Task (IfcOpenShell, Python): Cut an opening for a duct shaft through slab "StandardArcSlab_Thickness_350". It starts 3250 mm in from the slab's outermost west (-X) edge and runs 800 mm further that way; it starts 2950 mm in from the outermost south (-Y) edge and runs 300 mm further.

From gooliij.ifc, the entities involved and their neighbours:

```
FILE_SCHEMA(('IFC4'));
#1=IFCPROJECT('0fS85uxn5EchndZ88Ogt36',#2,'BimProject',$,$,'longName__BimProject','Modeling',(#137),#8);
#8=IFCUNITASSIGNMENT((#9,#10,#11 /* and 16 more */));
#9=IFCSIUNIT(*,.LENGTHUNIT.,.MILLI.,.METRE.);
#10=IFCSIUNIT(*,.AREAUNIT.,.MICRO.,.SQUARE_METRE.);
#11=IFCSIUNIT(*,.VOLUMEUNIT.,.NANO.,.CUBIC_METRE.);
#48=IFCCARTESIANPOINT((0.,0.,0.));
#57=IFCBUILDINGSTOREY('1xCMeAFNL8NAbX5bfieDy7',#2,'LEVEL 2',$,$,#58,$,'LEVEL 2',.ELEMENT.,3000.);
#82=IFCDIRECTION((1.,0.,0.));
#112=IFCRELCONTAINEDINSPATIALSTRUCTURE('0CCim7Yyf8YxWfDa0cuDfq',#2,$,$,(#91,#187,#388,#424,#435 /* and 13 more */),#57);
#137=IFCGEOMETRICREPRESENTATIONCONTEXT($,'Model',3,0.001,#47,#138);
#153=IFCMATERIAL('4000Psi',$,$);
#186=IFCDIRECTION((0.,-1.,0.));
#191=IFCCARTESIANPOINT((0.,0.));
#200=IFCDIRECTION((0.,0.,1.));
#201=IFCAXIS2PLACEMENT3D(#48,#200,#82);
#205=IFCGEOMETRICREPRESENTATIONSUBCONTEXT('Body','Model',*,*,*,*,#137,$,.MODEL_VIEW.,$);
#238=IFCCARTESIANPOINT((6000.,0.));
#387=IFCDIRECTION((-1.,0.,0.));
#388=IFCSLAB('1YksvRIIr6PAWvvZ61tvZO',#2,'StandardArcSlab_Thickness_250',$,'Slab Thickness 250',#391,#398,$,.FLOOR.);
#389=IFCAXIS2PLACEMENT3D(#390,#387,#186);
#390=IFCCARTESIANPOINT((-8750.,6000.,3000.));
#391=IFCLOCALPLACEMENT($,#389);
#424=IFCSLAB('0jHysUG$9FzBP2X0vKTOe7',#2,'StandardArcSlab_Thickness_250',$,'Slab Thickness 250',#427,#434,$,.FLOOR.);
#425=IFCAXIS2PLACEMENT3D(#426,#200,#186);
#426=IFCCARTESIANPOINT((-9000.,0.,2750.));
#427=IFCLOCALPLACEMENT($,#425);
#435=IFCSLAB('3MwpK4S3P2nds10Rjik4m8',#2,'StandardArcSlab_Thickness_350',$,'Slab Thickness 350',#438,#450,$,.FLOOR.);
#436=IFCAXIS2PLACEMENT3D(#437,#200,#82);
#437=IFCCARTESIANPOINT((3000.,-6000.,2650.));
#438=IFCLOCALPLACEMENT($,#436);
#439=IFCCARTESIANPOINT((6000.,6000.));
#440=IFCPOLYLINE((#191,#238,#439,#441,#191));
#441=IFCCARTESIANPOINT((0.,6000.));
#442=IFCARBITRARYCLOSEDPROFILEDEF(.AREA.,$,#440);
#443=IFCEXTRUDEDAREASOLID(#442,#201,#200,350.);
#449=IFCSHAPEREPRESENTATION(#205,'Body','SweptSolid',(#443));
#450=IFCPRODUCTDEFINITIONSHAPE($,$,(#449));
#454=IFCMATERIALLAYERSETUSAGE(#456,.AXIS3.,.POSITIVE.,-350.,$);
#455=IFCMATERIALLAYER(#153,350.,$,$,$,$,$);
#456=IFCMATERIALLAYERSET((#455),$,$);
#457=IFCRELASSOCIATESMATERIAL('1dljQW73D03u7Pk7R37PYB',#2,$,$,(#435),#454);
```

```python
import numpy as np
import ifcopenshell
import ifcopenshell.api.feature
import ifcopenshell.api.geometry
import ifcopenshell.api.root
import ifcopenshell.geom
import ifcopenshell.util.placement
import ifcopenshell.util.representation
import ifcopenshell.util.shape
import ifcopenshell.util.unit

model = ifcopenshell.open("gooliij.ifc")
unit_scale = ifcopenshell.util.unit.calculate_unit_scale(model)
settings = ifcopenshell.geom.settings()


def volume(element):
    """Net volume in cubic metres, openings subtracted."""
    shape = ifcopenshell.geom.create_shape(settings, element)
    return ifcopenshell.util.shape.get_volume(shape.geometry)


slab = model.by_guid("3MwpK4S3P2nds10Rjik4m8")
before = volume(slab)

# Extent in the slab's own axes, in metres. The edges named are its -X and -Y sides.
slab_shape = ifcopenshell.geom.create_shape(settings, slab)
vertices = ifcopenshell.util.shape.get_vertices(slab_shape.geometry)
x_min, y_min, bottom = vertices.min(axis=0)
top = vertices[:, 2].max()

opening = ifcopenshell.api.root.create_entity(model, ifc_class="IfcOpeningElement", name="Duct shaft opening", predefined_type="OPENING")
context = ifcopenshell.util.representation.get_context(model, "Model", "Body", "MODEL_VIEW")
width, depth = 0.8, 0.3
outline = [(0.0, 0.0), (width, 0.0), (width, depth), (0.0, depth), (0.0, 0.0)]
# Overshoot both faces by 50 mm so the cut is clean.
shape = ifcopenshell.api.geometry.add_slab_representation(
    model, context=context, depth=top - bottom + 0.1, polyline=outline
)
ifcopenshell.api.geometry.assign_representation(model, product=opening, representation=shape)

matrix = ifcopenshell.util.placement.get_local_placement(slab.ObjectPlacement)
matrix[:, 3] = matrix @ np.append(np.array([x_min + 3.25, y_min + 2.95, bottom - 0.05]) / unit_scale, 1.0)
ifcopenshell.api.geometry.edit_object_placement(model, product=opening, matrix=matrix, is_si=False)
ifcopenshell.api.feature.add_feature(model, feature=opening, element=slab)

after = volume(slab)

print(f"slab volume {before:.3f} -> {after:.3f} m3")

model.write("gooliij_rev.ifc")
```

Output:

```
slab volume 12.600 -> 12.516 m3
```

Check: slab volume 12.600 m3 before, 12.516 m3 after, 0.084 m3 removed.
